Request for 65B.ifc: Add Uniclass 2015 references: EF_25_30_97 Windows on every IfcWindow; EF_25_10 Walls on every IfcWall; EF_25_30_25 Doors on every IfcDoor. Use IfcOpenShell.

First a look at what the model holds.

```python
import ifcopenshell

model = ifcopenshell.open("65B.ifc")
print(model.schema)
print("classifications:", [c.Name for c in model.by_type("IfcClassification")])
for ifc_class in ("IfcDoor", "IfcRoof", "IfcStair", "IfcWall", "IfcWindow"):
    print(ifc_class, len(model.by_type(ifc_class)))
```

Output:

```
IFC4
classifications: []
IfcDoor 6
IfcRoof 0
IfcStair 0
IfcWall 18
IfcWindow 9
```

```python
import ifcopenshell
import ifcopenshell.api.classification

model = ifcopenshell.open("65B.ifc")

system = ifcopenshell.api.classification.add_classification(model, classification="Uniclass 2015")

codes = {
    "IfcWindow": ("EF_25_30_97", "Windows"),
    "IfcWall": ("EF_25_10", "Walls"),
    "IfcDoor": ("EF_25_30_25", "Doors"),
}
for ifc_class, (code, name) in codes.items():
    products = model.by_type(ifc_class)
    ifcopenshell.api.classification.add_reference(
        model, products=products, classification=system, identification=code, name=name
    )
    print(code, len(products))

model.write("65B-out.ifc")
```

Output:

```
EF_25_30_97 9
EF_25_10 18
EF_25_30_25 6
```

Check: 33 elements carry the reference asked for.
